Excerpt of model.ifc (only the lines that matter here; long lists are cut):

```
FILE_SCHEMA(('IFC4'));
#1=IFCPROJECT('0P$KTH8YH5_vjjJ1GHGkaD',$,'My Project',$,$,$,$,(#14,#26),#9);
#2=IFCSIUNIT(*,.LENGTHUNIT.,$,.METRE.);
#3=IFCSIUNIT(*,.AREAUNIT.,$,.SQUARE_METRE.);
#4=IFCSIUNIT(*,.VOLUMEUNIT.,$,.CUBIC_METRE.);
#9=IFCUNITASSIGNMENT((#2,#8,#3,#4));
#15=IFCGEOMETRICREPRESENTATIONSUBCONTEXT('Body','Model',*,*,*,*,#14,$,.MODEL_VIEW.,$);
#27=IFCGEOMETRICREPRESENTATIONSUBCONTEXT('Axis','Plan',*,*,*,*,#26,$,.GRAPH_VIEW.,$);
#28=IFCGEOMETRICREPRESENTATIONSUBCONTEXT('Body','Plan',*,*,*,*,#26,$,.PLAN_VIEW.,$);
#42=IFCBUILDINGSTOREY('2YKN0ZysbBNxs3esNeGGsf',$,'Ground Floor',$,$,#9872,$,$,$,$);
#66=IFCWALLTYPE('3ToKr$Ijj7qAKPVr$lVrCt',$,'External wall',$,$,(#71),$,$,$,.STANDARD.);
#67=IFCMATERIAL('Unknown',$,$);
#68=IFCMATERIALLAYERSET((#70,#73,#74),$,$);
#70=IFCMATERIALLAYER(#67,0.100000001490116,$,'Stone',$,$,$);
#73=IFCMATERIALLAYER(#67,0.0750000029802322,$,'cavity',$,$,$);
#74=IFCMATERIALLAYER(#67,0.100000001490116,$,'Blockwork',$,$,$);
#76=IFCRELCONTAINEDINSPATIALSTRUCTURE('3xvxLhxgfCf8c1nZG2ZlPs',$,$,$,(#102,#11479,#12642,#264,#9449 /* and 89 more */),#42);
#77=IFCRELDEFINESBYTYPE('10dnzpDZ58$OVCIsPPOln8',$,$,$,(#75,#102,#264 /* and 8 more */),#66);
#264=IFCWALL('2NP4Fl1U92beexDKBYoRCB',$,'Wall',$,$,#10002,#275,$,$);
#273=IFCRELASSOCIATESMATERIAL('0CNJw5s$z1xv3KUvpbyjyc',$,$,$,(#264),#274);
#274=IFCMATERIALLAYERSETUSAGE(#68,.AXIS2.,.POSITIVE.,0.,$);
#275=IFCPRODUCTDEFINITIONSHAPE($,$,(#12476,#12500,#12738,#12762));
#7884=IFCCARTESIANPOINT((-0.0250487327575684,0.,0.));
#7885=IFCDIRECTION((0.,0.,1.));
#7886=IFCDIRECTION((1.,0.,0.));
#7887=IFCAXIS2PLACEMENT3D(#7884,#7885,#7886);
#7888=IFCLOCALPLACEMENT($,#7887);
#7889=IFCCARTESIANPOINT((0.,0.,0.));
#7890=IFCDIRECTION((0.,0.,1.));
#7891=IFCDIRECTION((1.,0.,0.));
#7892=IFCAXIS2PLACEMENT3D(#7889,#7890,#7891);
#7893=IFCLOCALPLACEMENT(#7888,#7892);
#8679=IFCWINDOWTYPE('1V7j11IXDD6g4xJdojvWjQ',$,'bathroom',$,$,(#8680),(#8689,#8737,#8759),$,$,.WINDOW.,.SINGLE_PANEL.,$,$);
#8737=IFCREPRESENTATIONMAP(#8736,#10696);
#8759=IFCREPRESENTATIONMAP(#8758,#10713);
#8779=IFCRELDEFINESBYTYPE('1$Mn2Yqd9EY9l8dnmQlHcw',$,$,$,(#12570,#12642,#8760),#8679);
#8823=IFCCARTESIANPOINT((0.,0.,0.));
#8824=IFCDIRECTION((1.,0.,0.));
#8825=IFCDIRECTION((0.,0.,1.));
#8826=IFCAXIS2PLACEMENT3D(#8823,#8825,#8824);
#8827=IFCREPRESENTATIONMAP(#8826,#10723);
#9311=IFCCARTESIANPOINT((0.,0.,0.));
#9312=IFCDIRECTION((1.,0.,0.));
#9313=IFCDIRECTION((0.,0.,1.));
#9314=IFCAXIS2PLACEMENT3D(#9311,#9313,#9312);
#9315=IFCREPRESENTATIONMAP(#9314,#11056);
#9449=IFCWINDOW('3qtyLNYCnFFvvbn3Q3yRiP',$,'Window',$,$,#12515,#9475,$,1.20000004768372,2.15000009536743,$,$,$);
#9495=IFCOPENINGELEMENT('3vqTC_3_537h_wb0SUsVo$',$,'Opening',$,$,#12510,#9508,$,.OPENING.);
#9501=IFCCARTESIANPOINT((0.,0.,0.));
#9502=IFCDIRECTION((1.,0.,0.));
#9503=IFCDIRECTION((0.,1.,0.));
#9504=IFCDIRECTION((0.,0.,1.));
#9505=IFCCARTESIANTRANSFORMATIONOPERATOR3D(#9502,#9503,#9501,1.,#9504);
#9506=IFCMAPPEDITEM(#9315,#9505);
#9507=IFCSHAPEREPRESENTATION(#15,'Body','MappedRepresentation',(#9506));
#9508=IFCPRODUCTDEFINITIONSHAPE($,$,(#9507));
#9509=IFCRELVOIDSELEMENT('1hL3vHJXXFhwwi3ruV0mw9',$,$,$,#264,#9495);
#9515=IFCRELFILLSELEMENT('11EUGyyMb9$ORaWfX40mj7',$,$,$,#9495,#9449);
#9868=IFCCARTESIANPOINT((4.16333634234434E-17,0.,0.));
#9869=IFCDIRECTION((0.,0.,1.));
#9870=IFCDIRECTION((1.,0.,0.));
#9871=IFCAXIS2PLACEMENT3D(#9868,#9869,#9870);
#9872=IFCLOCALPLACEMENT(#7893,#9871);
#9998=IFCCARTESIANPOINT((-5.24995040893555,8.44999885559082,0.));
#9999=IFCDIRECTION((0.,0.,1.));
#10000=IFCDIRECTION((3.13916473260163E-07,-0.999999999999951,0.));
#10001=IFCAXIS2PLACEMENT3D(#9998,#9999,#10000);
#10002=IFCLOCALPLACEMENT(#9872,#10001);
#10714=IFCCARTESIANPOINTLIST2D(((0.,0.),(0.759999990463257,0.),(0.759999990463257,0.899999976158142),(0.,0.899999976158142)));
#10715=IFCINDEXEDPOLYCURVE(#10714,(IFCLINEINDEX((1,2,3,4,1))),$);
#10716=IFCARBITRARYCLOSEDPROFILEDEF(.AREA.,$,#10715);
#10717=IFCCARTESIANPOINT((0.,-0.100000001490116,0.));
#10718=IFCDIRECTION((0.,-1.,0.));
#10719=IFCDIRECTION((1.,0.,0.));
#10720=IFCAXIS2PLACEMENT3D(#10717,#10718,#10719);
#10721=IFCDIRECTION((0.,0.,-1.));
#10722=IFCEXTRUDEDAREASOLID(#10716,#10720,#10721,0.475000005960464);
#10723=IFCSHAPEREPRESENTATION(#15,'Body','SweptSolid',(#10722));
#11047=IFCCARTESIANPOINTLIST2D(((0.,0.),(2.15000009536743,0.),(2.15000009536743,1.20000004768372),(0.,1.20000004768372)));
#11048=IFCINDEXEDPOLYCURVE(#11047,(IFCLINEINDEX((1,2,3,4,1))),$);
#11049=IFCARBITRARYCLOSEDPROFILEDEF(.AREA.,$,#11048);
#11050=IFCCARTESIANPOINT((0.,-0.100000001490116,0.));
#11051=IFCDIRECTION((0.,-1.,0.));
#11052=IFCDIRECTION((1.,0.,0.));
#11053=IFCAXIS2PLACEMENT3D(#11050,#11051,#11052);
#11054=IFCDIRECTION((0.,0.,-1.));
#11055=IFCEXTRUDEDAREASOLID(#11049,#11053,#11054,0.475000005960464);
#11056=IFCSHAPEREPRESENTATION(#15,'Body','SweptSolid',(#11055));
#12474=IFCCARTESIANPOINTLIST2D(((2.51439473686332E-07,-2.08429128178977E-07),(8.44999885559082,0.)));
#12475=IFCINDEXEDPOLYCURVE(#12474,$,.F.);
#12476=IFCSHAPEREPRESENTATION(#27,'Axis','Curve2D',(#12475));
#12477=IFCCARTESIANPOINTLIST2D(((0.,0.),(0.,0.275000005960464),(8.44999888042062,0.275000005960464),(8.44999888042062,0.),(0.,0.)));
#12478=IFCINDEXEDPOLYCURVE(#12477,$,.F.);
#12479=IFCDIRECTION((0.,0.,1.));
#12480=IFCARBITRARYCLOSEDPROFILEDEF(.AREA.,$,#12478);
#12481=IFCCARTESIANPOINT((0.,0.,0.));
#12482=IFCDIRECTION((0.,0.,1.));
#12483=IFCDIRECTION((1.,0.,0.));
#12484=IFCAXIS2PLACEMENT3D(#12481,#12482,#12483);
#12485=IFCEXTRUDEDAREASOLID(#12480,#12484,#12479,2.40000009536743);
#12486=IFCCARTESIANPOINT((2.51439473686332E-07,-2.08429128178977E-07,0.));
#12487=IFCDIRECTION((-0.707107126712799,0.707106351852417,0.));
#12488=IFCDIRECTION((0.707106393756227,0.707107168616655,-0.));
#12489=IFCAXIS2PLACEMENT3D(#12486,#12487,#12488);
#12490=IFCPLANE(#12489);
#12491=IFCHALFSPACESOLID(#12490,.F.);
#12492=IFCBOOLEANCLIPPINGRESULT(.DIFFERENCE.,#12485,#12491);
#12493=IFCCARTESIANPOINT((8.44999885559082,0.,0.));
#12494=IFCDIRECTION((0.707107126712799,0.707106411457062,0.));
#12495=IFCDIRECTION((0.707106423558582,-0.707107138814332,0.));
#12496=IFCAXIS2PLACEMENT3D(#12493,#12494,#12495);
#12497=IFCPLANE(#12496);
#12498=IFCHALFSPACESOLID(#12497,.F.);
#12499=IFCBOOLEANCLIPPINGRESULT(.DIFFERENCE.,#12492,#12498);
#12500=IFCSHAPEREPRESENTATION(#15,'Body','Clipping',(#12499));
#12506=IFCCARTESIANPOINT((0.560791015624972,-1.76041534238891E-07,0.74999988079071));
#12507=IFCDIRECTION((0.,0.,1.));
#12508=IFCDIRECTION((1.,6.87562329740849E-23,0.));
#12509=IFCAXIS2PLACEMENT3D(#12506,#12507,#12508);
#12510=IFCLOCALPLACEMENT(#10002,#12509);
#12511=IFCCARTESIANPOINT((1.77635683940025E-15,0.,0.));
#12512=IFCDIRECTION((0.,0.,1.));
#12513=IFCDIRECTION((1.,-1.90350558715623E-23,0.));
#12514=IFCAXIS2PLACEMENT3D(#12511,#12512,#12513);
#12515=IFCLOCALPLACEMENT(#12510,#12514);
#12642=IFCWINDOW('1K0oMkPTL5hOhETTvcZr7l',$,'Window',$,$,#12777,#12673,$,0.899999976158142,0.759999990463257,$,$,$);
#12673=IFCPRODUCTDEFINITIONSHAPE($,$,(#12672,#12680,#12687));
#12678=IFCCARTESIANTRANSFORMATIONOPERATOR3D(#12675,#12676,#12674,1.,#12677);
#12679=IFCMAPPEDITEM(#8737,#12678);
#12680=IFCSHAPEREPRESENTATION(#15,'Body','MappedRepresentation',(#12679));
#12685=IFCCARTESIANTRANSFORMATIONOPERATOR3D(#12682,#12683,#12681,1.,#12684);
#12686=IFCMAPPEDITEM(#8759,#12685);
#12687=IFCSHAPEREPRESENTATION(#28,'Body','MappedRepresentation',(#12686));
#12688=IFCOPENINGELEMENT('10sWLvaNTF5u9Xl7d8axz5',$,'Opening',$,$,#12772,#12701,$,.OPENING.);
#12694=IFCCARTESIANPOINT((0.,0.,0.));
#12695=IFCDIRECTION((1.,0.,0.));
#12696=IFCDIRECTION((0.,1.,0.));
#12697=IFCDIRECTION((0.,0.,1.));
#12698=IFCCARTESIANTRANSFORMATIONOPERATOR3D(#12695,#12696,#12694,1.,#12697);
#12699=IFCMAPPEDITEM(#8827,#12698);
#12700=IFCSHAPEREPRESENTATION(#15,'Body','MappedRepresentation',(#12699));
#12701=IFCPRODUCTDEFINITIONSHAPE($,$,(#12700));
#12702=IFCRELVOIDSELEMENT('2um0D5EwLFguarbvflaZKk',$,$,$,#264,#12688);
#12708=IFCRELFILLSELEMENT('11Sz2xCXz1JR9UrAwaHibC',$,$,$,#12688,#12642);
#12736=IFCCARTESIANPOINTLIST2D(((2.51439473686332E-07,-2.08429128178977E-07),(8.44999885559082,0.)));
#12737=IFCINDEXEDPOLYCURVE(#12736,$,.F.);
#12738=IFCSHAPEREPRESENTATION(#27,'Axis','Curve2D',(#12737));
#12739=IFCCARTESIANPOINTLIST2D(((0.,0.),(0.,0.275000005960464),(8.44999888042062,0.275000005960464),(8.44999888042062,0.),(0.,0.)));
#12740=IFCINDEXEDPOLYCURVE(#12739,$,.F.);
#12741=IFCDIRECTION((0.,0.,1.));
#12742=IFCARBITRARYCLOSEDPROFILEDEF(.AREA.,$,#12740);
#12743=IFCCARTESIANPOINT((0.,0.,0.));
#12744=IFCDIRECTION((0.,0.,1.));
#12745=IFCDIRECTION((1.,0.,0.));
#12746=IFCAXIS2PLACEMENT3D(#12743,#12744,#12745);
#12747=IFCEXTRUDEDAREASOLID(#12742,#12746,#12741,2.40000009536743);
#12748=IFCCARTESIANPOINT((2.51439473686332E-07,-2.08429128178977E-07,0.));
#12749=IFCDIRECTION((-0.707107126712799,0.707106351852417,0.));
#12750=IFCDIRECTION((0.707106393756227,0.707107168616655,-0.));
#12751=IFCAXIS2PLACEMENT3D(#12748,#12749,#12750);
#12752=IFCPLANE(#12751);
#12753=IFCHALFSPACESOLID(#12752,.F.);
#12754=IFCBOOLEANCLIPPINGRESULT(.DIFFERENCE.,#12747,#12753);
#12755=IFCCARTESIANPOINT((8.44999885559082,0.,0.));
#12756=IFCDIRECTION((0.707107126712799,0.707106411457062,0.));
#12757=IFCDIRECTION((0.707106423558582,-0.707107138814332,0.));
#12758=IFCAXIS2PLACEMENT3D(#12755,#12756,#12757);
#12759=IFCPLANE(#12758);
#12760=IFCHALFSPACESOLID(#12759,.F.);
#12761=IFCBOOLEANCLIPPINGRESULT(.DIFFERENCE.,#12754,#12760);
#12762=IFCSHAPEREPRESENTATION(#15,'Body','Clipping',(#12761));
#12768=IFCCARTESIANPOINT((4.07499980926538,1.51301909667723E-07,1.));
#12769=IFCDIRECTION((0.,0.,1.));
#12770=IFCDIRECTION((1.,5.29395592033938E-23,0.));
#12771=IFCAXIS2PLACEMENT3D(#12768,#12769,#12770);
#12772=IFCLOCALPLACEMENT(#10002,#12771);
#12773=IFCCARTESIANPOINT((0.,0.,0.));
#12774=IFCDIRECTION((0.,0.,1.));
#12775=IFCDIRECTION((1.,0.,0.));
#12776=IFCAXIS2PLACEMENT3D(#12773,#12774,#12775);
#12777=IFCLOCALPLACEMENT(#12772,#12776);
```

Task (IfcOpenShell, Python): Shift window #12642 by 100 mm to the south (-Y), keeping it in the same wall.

```python
import ifcopenshell
import ifcopenshell.api.geometry
import ifcopenshell.util.placement
import ifcopenshell.util.unit

model = ifcopenshell.open("model.ifc")
unit_scale = ifcopenshell.util.unit.calculate_unit_scale(model)

window = model.by_guid("1K0oMkPTL5hOhETTvcZr7l")
opening = window.FillsVoids[0].RelatingOpeningElement
wall = opening.VoidsElements[0].RelatingBuildingElement

wall_matrix = ifcopenshell.util.placement.get_local_placement(wall.ObjectPlacement)
shift = wall_matrix[:3, 0] * 0.1 / unit_scale
before = ifcopenshell.util.placement.get_local_placement(window.ObjectPlacement)[:3, 3].copy()

# The window is placed relative to its opening, so it follows when the opening moves.
matrix = ifcopenshell.util.placement.get_local_placement(opening.ObjectPlacement)
matrix[:3, 3] += shift
ifcopenshell.api.geometry.edit_object_placement(
    model, product=opening, matrix=matrix, is_si=False, should_transform_children=True
)

after = ifcopenshell.util.placement.get_local_placement(window.ObjectPlacement)[:3, 3]
print("window moved by", (after - before).round(3) + 0.0)

model.write("model_rev.ifc")
```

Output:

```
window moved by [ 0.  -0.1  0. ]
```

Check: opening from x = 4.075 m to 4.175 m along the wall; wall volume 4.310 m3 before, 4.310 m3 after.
